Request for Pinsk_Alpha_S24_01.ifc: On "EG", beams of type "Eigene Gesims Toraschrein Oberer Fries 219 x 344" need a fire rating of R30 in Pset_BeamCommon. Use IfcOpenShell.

First a look at what the model holds.

```python
import ifcopenshell
import ifcopenshell.util.element

model = ifcopenshell.open("Pinsk_Alpha_S24_01.ifc")
print(model.schema)
storey = next(s for s in model.by_type("IfcBuildingStorey") if s.Name == "EG")
beams = [e for e in ifcopenshell.util.element.get_decomposition(storey) if e.is_a("IfcBeam")]
seen = {}
for e in beams:
    element_type = ifcopenshell.util.element.get_type(e)
    key = (element_type.Name if element_type != e and element_type else None, ifcopenshell.util.element.get_pset(e, "Pset_BeamCommon", "FireRating"))
    seen[key] = seen.get(key, 0) + 1
for (name, value), count in sorted(seen.items(), key=str):
    print(count, "x", name, "|", value)
```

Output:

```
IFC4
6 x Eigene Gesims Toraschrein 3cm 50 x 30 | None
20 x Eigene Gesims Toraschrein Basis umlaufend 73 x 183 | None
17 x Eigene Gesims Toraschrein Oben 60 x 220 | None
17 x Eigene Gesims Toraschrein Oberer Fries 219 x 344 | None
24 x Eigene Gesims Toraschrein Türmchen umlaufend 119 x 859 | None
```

```python
import ifcopenshell
import ifcopenshell.api.pset
import ifcopenshell.util.element

model = ifcopenshell.open("Pinsk_Alpha_S24_01.ifc")

storey = next(s for s in model.by_type("IfcBuildingStorey") if s.Name == "EG")
beams = [e for e in ifcopenshell.util.element.get_decomposition(storey) if e.is_a("IfcBeam")]

count = 0
for e in beams:
    element_type = ifcopenshell.util.element.get_type(e)
    if element_type in (None, e) or element_type.Name != "Eigene Gesims Toraschrein Oberer Fries 219 x 344":
        continue
    # add_pset returns the element's existing set when there is one.
    pset = ifcopenshell.api.pset.add_pset(model, product=e, name="Pset_BeamCommon")
    ifcopenshell.api.pset.edit_pset(model, pset=pset, properties={"FireRating": "R30"})
    count += 1

print(count, "beams updated")

model.write("Pinsk_Alpha_S24_01_rev.ifc")
```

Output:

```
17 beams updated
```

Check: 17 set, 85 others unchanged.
